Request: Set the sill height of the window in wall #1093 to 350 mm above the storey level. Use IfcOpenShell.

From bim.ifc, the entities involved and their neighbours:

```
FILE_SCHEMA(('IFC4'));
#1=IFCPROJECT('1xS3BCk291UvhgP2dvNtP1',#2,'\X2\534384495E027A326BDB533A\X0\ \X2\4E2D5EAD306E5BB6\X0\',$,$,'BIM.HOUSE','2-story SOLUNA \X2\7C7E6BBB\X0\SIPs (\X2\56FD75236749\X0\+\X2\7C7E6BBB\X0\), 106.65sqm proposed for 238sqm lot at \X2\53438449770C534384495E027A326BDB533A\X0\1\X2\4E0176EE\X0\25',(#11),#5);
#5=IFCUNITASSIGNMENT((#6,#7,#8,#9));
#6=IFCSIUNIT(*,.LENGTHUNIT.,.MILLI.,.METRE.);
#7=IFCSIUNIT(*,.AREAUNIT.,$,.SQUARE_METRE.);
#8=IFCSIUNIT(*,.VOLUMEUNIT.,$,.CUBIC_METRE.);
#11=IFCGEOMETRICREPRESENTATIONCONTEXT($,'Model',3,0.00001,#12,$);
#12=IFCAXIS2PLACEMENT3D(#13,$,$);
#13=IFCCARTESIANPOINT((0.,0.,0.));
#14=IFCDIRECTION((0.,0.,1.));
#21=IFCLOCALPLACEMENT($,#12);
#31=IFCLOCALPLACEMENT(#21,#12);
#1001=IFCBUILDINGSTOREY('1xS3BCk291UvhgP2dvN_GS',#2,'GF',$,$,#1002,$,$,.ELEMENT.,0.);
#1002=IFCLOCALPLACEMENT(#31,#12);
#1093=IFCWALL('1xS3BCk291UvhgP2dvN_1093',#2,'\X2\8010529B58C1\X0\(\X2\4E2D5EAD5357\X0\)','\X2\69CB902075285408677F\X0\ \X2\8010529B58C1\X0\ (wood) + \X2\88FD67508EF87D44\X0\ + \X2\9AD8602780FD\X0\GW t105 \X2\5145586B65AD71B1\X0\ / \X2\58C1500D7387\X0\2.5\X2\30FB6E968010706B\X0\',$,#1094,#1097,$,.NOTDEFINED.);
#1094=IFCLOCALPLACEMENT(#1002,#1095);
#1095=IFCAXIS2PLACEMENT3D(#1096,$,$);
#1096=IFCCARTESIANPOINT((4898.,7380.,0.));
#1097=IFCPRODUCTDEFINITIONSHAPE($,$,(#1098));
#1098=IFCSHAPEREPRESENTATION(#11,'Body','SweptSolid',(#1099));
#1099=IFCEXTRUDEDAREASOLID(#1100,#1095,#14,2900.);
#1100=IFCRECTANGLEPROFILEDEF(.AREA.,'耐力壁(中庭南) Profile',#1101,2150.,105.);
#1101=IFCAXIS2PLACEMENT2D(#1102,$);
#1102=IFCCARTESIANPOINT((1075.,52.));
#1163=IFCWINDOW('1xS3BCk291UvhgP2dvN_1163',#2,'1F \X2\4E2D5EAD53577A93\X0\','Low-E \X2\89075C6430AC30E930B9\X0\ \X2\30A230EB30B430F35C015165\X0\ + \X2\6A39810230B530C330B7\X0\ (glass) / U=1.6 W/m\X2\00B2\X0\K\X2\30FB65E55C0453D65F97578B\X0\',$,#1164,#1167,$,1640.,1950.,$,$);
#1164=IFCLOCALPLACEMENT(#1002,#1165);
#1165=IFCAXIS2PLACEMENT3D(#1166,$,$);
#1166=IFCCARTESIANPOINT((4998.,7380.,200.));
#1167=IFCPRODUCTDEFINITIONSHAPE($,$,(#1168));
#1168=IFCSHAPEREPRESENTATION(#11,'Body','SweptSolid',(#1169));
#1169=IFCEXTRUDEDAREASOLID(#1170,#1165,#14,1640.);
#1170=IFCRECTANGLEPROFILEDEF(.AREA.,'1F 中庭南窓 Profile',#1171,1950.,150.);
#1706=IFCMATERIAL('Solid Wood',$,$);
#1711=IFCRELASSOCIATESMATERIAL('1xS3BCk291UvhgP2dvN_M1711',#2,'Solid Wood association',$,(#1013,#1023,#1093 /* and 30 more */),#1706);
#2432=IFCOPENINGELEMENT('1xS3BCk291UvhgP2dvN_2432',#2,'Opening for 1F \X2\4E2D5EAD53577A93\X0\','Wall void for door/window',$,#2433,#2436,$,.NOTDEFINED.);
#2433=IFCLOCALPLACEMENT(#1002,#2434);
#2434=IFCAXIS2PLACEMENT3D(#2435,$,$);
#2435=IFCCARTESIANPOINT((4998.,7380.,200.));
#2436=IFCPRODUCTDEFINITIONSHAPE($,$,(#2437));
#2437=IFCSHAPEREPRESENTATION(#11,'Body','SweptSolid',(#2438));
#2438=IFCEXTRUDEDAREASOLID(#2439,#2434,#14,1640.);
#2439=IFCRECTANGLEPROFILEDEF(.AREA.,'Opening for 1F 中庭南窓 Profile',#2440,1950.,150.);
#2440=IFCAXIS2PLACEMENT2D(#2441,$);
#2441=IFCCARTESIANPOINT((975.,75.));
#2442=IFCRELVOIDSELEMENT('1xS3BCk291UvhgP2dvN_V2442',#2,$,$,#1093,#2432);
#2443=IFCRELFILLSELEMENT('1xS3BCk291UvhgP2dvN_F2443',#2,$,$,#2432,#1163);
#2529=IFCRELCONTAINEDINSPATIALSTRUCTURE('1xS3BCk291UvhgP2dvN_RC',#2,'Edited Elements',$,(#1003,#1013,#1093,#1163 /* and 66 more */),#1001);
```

```python
import numpy as np
import ifcopenshell
import ifcopenshell.api.geometry
import ifcopenshell.geom
import ifcopenshell.util.element
import ifcopenshell.util.placement
import ifcopenshell.util.shape
import ifcopenshell.util.unit

model = ifcopenshell.open("bim.ifc")
unit_scale = ifcopenshell.util.unit.calculate_unit_scale(model)

window = model.by_guid("1xS3BCk291UvhgP2dvN_1163")
opening = window.FillsVoids[0].RelatingOpeningElement
storey = ifcopenshell.util.element.get_container(window, ifc_class="IfcBuildingStorey")
level = ifcopenshell.util.placement.get_local_placement(storey.ObjectPlacement)[2, 3]

# The opening's origin need not be at the sill, so measure its lowest point.
shape = ifcopenshell.geom.create_shape(ifcopenshell.geom.settings(), opening)
bottom = ifcopenshell.util.shape.get_shape_bottom_elevation(shape, shape.geometry) / unit_scale
dz = level + 350.0 - bottom

shift = np.array([0.0, 0.0, dz])
# The window is not placed relative to its opening, so move both.
for product in (opening, window):
    matrix = ifcopenshell.util.placement.get_local_placement(product.ObjectPlacement)
    matrix[:3, 3] += shift
    ifcopenshell.api.geometry.edit_object_placement(model, product=product, matrix=matrix, is_si=False)

print(f"moved by {dz * unit_scale:+.3f} m")

model.write("bim_updated.ifc")
```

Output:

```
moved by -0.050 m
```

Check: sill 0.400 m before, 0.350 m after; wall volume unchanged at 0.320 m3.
